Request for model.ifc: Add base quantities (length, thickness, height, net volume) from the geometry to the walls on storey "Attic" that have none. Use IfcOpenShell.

First a look at what the model holds.

```python
import ifcopenshell
import ifcopenshell.util.element
import ifcopenshell.util.unit

model = ifcopenshell.open("model.ifc")
print(model.schema)
for unit_type in ("LENGTHUNIT", "AREAUNIT", "VOLUMEUNIT"):
    print(unit_type, ifcopenshell.util.unit.calculate_unit_scale(model, unit_type))
storey = next(s for s in model.by_type("IfcBuildingStorey") if s.Name == "Attic")
walls = [e for e in ifcopenshell.util.element.get_decomposition(storey) if e.is_a("IfcWall")]
for e in sorted(walls, key=lambda e: e.id()):
    print(e.id(), e.is_a(), e.Name, list(ifcopenshell.util.element.get_psets(e, qtos_only=True)), sep=" | ")
```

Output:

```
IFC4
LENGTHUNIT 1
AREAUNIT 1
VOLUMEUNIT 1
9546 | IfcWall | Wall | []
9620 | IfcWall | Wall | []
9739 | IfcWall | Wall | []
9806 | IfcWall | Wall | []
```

```python
import ifcopenshell
import ifcopenshell.api.pset
import ifcopenshell.geom
import ifcopenshell.util.element
import ifcopenshell.util.shape
import ifcopenshell.util.unit

model = ifcopenshell.open("model.ifc")
unit_scale = ifcopenshell.util.unit.calculate_unit_scale(model)
volume_scale = ifcopenshell.util.unit.calculate_unit_scale(model, "VOLUMEUNIT")
settings = ifcopenshell.geom.settings()

storey = next(s for s in model.by_type("IfcBuildingStorey") if s.Name == "Attic")
walls = [e for e in ifcopenshell.util.element.get_decomposition(storey) if e.is_a("IfcWall")]

for e in sorted(walls, key=lambda e: e.id()):
    if ifcopenshell.util.element.get_psets(e, qtos_only=True, should_inherit=False):
        continue
    # Geometry comes back in metres, in the element's own axes.
    shape = ifcopenshell.geom.create_shape(settings, e)
    values = {
        "Length": ifcopenshell.util.shape.get_x(shape.geometry) / unit_scale,
        "Width": ifcopenshell.util.shape.get_y(shape.geometry) / unit_scale,
        "Height": ifcopenshell.util.shape.get_z(shape.geometry) / unit_scale,
        "NetVolume": ifcopenshell.util.shape.get_volume(shape.geometry) / volume_scale,
    }
    qto = ifcopenshell.api.pset.add_qto(model, product=e, name="Qto_WallBaseQuantities")
    ifcopenshell.api.pset.edit_qto(model, qto=qto, properties=values)
    print(e.id(), {k: round(v, 3) for k, v in values.items()})

model.write("model_rev.ifc")
```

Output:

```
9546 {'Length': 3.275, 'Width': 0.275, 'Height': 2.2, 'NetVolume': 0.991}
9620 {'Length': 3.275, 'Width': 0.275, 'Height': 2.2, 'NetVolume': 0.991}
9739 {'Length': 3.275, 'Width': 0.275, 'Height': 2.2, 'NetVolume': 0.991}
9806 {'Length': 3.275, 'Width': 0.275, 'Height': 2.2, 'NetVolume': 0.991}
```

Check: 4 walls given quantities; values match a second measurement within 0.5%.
